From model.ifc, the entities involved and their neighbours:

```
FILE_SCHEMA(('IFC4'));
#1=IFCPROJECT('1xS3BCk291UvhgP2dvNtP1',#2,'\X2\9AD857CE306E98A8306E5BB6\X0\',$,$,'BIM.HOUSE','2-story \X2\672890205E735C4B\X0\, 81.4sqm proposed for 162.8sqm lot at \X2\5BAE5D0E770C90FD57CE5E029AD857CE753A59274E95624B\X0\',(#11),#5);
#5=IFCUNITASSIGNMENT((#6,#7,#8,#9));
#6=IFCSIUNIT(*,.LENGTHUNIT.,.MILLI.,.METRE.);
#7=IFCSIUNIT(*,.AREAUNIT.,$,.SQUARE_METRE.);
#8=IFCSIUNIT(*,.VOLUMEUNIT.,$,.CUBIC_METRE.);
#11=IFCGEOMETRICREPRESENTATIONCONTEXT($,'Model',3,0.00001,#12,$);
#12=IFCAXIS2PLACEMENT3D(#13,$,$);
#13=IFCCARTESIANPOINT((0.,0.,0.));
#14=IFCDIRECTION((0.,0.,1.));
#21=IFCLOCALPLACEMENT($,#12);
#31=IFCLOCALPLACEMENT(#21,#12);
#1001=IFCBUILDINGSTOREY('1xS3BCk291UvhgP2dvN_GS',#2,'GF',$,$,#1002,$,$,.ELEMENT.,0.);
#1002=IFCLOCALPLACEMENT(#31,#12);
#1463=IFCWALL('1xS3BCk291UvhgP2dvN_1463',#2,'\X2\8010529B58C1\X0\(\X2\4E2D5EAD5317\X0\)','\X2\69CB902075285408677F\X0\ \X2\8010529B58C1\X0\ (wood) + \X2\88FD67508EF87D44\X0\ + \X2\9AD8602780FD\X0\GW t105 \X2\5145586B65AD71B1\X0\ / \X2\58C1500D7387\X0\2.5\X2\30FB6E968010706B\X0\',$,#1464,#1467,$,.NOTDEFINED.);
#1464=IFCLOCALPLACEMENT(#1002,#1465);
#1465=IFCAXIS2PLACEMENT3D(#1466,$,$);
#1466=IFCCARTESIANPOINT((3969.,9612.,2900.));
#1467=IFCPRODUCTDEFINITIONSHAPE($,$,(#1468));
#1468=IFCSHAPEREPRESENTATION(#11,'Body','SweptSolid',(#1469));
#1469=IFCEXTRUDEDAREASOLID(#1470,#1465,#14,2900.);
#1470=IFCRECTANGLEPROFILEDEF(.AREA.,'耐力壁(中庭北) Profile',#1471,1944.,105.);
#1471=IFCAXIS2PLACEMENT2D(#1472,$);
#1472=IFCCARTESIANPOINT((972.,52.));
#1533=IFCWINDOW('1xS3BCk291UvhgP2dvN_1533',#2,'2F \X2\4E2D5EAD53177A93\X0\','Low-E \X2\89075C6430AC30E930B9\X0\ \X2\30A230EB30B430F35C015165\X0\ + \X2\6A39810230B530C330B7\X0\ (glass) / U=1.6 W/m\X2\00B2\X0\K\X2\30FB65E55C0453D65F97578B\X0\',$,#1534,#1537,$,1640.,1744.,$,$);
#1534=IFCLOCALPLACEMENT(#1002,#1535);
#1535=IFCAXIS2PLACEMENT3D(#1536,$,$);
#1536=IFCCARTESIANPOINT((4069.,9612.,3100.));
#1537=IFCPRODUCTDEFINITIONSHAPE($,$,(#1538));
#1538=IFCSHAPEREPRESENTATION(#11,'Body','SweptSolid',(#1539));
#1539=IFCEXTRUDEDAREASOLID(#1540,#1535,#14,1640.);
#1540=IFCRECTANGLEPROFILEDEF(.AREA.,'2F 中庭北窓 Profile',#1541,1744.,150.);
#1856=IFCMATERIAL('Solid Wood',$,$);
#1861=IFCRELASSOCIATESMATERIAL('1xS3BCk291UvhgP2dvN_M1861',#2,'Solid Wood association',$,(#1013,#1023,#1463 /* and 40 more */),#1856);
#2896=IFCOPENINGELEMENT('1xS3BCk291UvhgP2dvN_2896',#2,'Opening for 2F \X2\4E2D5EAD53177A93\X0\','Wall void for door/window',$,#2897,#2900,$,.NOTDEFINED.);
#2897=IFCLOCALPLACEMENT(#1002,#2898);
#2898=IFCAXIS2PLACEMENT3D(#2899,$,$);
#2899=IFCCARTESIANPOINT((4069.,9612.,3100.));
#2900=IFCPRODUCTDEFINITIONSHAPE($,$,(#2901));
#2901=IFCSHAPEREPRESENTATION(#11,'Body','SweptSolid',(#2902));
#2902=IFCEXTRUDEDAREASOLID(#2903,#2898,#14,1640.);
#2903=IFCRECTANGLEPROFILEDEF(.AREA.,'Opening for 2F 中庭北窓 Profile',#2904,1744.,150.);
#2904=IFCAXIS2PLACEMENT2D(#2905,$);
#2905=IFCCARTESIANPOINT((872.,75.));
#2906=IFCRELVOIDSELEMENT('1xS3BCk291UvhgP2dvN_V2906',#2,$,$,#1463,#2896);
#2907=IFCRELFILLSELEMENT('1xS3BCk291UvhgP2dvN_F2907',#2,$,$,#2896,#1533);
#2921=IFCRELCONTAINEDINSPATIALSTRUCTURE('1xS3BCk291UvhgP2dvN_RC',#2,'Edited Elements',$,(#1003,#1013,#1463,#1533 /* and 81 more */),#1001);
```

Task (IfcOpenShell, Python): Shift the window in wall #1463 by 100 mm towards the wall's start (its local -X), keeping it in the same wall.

```python
import ifcopenshell
import ifcopenshell.api.geometry
import ifcopenshell.util.placement
import ifcopenshell.util.unit

model = ifcopenshell.open("model.ifc")
unit_scale = ifcopenshell.util.unit.calculate_unit_scale(model)

window = model.by_guid("1xS3BCk291UvhgP2dvN_1533")
opening = window.FillsVoids[0].RelatingOpeningElement
wall = opening.VoidsElements[0].RelatingBuildingElement

wall_matrix = ifcopenshell.util.placement.get_local_placement(wall.ObjectPlacement)
shift = wall_matrix[:3, 0] * -0.1 / unit_scale
before = ifcopenshell.util.placement.get_local_placement(window.ObjectPlacement)[:3, 3].copy()

# The window is not placed relative to its opening, so move both.
for product in (opening, window):
    matrix = ifcopenshell.util.placement.get_local_placement(product.ObjectPlacement)
    matrix[:3, 3] += shift
    ifcopenshell.api.geometry.edit_object_placement(model, product=product, matrix=matrix, is_si=False)

after = ifcopenshell.util.placement.get_local_placement(window.ObjectPlacement)[:3, 3]
print("window moved by", (after - before).round(3) + 0.0)

model.write("model_rev.ifc")
```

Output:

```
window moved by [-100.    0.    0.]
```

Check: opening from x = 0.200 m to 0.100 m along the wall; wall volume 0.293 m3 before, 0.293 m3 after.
